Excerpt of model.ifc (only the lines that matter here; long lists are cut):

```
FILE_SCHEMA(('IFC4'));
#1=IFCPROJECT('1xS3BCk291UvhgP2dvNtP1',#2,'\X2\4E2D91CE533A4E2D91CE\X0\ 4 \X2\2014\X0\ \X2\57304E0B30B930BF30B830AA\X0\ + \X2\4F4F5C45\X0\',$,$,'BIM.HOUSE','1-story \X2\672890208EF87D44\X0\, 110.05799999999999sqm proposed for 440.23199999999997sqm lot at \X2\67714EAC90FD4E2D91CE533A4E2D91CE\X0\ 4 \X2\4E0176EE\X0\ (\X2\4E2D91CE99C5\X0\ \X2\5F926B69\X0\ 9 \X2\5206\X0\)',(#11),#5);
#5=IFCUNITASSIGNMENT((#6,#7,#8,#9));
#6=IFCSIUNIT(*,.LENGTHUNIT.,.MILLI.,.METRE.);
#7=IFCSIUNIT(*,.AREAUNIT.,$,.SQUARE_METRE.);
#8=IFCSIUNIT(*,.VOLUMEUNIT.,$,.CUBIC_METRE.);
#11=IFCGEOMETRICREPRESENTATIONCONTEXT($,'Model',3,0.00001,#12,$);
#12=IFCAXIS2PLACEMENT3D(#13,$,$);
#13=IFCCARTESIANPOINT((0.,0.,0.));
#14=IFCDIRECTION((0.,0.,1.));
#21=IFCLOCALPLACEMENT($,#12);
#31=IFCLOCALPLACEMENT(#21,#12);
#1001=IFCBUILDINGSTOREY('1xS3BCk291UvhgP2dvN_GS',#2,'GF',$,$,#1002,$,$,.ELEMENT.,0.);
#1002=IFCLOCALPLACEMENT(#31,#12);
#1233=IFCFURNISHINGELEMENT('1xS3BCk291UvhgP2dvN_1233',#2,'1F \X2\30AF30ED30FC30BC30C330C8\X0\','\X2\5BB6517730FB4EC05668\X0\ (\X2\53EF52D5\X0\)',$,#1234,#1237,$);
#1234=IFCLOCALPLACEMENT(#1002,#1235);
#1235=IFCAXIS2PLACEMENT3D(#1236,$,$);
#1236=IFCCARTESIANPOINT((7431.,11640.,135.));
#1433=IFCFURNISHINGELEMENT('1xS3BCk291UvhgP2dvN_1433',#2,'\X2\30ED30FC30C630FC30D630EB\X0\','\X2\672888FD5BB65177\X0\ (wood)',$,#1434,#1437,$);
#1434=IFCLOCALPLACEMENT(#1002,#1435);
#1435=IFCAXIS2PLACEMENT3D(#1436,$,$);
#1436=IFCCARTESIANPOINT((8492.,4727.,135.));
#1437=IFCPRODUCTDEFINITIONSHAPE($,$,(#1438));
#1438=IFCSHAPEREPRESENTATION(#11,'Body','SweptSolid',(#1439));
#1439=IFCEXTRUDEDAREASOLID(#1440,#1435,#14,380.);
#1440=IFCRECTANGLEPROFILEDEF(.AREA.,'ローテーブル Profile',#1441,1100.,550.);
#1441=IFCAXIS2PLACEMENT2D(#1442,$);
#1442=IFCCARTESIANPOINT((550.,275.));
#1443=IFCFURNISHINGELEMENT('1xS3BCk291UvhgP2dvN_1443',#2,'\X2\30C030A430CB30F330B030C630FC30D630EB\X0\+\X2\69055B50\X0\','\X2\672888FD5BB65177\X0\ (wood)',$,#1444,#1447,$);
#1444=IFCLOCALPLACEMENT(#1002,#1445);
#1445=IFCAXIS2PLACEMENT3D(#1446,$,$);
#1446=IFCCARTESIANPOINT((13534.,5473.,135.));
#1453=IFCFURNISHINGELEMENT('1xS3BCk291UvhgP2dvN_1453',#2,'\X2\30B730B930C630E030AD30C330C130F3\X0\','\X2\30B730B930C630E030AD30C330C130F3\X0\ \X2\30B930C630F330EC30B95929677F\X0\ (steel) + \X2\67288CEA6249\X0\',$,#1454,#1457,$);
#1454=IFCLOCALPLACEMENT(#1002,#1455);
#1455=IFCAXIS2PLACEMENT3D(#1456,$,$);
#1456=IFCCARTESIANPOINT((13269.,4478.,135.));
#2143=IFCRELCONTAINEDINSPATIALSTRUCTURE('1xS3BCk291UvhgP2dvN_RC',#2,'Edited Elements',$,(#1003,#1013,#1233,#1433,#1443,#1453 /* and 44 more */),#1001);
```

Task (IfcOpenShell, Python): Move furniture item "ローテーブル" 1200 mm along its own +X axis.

```python
import ifcopenshell
import ifcopenshell.api.geometry
import ifcopenshell.util.placement

model = ifcopenshell.open("model.ifc")

item = model.by_id(1433)
matrix = ifcopenshell.util.placement.get_local_placement(item.ObjectPlacement)
matrix[:3, 3] += matrix[:3, 0] * 1200.0
ifcopenshell.api.geometry.edit_object_placement(model, product=item, matrix=matrix, is_si=False)

print(ifcopenshell.util.placement.get_local_placement(item.ObjectPlacement).round(3) + 0.0)

model.write("model_edited.ifc")
```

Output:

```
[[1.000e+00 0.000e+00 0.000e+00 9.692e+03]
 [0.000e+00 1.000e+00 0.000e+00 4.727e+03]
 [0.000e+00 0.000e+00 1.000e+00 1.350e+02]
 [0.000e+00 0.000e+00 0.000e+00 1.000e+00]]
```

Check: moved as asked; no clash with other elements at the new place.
